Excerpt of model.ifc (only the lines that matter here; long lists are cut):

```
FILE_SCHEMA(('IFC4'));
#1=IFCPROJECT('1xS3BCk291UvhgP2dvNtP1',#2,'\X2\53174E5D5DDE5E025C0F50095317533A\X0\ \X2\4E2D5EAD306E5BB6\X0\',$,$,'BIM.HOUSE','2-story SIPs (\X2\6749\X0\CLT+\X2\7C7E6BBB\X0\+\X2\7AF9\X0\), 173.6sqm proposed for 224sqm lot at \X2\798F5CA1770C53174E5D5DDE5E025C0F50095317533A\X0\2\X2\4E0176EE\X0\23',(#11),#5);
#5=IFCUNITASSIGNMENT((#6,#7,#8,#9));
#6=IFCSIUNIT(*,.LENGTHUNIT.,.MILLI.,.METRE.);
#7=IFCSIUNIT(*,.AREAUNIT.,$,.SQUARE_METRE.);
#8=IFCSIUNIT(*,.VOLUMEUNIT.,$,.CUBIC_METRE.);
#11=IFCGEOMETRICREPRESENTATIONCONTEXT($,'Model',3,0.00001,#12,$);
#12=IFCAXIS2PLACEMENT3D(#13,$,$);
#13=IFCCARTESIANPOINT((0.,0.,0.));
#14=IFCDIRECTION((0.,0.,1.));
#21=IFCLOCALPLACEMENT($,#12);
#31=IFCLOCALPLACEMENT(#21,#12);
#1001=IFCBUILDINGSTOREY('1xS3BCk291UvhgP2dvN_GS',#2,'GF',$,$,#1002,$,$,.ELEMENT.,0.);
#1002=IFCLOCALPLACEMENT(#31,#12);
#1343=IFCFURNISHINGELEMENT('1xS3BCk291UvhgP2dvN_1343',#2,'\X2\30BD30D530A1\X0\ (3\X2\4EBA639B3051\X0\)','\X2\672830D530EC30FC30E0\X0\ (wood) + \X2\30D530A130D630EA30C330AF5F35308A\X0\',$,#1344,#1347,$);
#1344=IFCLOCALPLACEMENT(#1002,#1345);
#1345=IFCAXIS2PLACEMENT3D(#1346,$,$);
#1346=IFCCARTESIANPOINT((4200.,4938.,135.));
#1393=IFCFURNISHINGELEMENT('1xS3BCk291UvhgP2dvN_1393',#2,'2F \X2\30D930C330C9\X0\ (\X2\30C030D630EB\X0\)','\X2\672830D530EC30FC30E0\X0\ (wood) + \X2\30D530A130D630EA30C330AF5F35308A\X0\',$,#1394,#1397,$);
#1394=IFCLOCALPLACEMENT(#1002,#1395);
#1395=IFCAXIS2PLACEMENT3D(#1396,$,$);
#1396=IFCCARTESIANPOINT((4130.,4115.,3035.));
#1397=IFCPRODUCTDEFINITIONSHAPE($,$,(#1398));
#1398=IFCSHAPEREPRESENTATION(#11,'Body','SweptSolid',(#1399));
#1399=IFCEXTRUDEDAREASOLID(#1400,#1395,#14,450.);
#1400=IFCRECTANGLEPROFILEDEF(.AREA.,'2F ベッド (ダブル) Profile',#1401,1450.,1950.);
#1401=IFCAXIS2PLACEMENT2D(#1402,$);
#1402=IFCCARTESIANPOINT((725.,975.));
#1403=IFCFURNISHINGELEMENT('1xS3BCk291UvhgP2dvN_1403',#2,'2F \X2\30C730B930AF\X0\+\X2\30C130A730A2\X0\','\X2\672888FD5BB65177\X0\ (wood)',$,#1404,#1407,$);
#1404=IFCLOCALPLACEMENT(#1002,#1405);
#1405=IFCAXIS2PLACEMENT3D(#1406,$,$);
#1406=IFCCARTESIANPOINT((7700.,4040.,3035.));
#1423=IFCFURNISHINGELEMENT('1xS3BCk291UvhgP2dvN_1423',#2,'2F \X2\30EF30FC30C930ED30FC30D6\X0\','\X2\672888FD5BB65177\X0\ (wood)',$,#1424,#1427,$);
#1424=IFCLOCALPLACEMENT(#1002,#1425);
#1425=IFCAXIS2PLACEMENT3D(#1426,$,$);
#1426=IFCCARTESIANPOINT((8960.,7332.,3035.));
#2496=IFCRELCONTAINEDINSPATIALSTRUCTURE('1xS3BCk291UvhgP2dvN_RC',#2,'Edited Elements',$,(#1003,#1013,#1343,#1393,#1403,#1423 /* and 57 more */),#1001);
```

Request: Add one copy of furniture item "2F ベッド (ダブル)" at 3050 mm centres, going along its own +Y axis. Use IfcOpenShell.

```python
import ifcopenshell
import ifcopenshell.api.geometry
import ifcopenshell.api.root
import ifcopenshell.util.element
import ifcopenshell.util.placement

model = ifcopenshell.open("model.ifc")


def reuse_history(source, copy):
    """copy_class also copies each property set's owner history, people and application; keep the originals."""
    for rel in copy.IsDefinedBy:
        if rel.is_a("IfcRelDefinesByProperties") and (history := rel.RelatingPropertyDefinition.OwnerHistory):
            rel.RelatingPropertyDefinition.OwnerHistory = source.OwnerHistory
            ifcopenshell.util.element.remove_deep2(model, history)


source = model.by_guid("1xS3BCk291UvhgP2dvN_1393")
base = ifcopenshell.util.placement.get_local_placement(source.ObjectPlacement)
step = base[:3, 1] * 3050.0

for i in range(1, 2):
    copy = ifcopenshell.api.root.copy_class(model, product=source)
    copy.Representation = ifcopenshell.util.element.copy_deep(
        model, source.Representation, exclude=["IfcGeometricRepresentationContext", "IfcRepresentationMap"]
    )
    reuse_history(source, copy)
    matrix = base.copy()
    matrix[:3, 3] += i * step
    print("added at", matrix[:3, 3].round(3) + 0.0)
    ifcopenshell.api.geometry.edit_object_placement(model, product=copy, matrix=matrix, is_si=False)

model.write("model_updated.ifc")
```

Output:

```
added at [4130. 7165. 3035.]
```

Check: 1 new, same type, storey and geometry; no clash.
